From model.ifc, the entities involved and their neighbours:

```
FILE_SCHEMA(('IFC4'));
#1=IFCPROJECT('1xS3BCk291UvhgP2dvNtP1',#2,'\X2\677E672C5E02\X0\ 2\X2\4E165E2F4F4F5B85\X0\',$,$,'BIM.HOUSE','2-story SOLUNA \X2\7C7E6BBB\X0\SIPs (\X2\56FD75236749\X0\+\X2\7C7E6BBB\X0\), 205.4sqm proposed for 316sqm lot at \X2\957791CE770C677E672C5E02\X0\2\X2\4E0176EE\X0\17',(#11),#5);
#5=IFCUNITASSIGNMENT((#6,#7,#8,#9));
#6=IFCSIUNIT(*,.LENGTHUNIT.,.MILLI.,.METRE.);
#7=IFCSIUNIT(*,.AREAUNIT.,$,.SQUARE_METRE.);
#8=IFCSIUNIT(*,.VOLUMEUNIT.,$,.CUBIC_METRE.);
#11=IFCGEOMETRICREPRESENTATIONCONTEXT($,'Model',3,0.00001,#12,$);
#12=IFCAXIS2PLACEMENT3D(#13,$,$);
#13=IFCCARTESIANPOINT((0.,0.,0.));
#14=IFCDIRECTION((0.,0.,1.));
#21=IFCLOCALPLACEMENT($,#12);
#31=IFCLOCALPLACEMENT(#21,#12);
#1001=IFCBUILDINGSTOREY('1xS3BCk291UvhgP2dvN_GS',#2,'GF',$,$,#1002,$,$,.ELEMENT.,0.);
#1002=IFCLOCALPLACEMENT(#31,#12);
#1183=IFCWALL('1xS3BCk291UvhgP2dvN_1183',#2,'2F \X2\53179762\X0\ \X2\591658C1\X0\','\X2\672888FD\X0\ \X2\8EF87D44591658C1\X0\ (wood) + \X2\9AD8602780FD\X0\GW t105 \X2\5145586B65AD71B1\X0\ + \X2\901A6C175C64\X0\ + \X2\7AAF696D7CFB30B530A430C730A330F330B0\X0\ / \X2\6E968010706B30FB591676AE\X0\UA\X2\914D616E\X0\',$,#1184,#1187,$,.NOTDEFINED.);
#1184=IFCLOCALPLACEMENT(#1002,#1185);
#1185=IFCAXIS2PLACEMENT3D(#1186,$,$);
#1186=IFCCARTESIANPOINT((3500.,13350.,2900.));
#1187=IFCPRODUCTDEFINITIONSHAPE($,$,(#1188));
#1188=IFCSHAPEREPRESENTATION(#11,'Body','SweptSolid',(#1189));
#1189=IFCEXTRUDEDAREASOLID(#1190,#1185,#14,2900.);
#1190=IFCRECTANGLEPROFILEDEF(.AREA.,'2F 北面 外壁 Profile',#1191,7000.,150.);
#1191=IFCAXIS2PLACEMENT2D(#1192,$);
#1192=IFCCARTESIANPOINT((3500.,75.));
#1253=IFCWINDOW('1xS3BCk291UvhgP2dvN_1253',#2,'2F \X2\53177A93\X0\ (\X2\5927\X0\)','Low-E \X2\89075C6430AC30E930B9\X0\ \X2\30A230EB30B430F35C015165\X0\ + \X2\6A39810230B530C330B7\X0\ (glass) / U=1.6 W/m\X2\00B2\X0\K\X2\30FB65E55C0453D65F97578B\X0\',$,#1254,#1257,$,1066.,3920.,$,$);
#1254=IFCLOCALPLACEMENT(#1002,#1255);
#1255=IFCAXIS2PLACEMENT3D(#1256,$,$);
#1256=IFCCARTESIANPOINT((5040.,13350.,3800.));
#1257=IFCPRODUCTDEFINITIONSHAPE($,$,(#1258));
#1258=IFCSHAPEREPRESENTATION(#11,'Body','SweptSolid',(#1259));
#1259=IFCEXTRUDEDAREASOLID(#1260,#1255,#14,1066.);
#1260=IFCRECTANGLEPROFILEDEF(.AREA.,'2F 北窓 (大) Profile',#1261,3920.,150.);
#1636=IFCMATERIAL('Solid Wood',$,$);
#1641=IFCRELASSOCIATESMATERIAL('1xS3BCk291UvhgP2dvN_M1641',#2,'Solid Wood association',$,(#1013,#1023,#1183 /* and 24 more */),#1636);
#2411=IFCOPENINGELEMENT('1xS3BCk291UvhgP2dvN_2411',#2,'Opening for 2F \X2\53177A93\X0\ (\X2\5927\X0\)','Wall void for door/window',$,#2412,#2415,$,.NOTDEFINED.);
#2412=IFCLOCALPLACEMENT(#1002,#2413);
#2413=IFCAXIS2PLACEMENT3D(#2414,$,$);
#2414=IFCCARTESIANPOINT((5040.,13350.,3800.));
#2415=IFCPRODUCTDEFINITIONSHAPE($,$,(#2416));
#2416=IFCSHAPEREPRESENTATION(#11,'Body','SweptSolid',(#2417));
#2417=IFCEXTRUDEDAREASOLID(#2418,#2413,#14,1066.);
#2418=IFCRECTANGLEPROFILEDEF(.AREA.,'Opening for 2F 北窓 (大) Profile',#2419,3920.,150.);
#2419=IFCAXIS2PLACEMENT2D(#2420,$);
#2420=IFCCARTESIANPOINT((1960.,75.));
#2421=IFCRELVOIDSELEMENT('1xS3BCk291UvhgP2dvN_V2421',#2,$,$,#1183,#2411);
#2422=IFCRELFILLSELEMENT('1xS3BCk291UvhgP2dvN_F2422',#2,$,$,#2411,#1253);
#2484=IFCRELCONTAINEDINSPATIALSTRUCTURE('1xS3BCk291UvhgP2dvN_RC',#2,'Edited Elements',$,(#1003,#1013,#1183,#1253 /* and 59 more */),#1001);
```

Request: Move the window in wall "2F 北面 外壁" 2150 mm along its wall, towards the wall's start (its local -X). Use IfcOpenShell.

```python
import ifcopenshell
import ifcopenshell.api.geometry
import ifcopenshell.util.placement
import ifcopenshell.util.unit

model = ifcopenshell.open("model.ifc")
unit_scale = ifcopenshell.util.unit.calculate_unit_scale(model)

window = model.by_id(1253)
opening = window.FillsVoids[0].RelatingOpeningElement
wall = opening.VoidsElements[0].RelatingBuildingElement

wall_matrix = ifcopenshell.util.placement.get_local_placement(wall.ObjectPlacement)
shift = wall_matrix[:3, 0] * -2.15 / unit_scale
before = ifcopenshell.util.placement.get_local_placement(window.ObjectPlacement)[:3, 3].copy()

# The window is not placed relative to its opening, so move both.
for product in (opening, window):
    matrix = ifcopenshell.util.placement.get_local_placement(product.ObjectPlacement)
    matrix[:3, 3] += shift
    ifcopenshell.api.geometry.edit_object_placement(model, product=product, matrix=matrix, is_si=False)

after = ifcopenshell.util.placement.get_local_placement(window.ObjectPlacement)[:3, 3]
print("window moved by", (after - before).round(3) + 0.0)

model.write("model_v2.ifc")
```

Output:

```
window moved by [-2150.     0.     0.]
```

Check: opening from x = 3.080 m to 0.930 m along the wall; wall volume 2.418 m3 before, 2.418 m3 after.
